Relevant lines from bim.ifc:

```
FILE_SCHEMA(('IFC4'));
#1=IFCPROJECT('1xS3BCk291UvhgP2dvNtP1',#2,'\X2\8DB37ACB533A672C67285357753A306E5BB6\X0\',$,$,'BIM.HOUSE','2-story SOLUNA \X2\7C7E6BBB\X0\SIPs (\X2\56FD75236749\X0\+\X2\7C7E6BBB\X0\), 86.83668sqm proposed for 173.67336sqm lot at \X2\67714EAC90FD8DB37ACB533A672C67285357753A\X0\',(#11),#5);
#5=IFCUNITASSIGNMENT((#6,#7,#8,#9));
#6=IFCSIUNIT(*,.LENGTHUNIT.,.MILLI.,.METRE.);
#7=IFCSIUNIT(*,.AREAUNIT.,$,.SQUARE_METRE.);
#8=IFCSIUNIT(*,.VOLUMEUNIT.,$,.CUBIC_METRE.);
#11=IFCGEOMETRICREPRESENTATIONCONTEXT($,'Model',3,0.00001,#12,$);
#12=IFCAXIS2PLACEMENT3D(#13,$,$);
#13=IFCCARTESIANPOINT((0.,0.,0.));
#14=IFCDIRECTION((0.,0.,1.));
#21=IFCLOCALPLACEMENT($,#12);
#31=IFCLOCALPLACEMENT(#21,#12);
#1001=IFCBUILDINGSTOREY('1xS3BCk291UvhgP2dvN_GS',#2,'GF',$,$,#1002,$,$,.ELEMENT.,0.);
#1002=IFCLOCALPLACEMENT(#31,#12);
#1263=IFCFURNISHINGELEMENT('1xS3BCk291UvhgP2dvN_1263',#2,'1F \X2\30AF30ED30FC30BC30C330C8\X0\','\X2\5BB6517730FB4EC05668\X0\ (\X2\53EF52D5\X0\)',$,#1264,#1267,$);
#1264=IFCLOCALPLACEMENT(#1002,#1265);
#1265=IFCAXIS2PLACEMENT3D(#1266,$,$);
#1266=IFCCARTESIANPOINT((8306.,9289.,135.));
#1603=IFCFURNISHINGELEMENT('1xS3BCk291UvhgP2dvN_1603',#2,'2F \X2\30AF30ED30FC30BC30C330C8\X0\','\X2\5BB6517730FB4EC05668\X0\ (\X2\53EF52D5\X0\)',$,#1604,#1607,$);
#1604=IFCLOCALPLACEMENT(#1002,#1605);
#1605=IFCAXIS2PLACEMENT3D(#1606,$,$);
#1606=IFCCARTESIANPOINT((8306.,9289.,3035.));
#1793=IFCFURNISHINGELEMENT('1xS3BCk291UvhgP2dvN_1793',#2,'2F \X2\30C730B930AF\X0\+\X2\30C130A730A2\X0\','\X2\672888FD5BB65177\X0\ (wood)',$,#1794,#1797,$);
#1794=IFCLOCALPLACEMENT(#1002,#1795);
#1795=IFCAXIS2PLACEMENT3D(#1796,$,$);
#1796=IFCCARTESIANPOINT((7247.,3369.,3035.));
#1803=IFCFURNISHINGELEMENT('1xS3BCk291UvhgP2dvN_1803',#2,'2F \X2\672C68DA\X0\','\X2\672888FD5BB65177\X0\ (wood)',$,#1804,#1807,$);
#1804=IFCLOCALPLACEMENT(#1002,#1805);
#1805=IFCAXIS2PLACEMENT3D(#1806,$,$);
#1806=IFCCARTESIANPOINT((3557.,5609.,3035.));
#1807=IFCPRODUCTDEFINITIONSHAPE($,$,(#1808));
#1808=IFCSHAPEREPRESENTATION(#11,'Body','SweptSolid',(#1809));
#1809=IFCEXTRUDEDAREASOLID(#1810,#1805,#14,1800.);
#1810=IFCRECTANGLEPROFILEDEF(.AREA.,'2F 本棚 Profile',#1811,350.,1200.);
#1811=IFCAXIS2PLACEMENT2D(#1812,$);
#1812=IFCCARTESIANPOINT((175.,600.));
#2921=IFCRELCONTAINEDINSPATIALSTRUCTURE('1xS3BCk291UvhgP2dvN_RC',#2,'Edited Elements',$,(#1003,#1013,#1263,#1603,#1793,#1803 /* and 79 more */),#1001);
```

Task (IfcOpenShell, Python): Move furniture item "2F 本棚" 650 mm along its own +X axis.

```python
import ifcopenshell
import ifcopenshell.api.geometry
import ifcopenshell.util.placement
import ifcopenshell.util.unit

model = ifcopenshell.open("bim.ifc")
unit_scale = ifcopenshell.util.unit.calculate_unit_scale(model)

item = model.by_guid("1xS3BCk291UvhgP2dvN_1803")
matrix = ifcopenshell.util.placement.get_local_placement(item.ObjectPlacement)
matrix[:3, 3] += matrix[:3, 0] * 0.65 / unit_scale
ifcopenshell.api.geometry.edit_object_placement(model, product=item, matrix=matrix, is_si=False)

print(ifcopenshell.util.placement.get_local_placement(item.ObjectPlacement).round(3) + 0.0)

model.write("bim_edited.ifc")
```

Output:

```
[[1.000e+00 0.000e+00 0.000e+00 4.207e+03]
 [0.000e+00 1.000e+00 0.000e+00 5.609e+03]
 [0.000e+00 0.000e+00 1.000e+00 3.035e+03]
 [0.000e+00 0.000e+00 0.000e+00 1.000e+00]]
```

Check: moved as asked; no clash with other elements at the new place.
